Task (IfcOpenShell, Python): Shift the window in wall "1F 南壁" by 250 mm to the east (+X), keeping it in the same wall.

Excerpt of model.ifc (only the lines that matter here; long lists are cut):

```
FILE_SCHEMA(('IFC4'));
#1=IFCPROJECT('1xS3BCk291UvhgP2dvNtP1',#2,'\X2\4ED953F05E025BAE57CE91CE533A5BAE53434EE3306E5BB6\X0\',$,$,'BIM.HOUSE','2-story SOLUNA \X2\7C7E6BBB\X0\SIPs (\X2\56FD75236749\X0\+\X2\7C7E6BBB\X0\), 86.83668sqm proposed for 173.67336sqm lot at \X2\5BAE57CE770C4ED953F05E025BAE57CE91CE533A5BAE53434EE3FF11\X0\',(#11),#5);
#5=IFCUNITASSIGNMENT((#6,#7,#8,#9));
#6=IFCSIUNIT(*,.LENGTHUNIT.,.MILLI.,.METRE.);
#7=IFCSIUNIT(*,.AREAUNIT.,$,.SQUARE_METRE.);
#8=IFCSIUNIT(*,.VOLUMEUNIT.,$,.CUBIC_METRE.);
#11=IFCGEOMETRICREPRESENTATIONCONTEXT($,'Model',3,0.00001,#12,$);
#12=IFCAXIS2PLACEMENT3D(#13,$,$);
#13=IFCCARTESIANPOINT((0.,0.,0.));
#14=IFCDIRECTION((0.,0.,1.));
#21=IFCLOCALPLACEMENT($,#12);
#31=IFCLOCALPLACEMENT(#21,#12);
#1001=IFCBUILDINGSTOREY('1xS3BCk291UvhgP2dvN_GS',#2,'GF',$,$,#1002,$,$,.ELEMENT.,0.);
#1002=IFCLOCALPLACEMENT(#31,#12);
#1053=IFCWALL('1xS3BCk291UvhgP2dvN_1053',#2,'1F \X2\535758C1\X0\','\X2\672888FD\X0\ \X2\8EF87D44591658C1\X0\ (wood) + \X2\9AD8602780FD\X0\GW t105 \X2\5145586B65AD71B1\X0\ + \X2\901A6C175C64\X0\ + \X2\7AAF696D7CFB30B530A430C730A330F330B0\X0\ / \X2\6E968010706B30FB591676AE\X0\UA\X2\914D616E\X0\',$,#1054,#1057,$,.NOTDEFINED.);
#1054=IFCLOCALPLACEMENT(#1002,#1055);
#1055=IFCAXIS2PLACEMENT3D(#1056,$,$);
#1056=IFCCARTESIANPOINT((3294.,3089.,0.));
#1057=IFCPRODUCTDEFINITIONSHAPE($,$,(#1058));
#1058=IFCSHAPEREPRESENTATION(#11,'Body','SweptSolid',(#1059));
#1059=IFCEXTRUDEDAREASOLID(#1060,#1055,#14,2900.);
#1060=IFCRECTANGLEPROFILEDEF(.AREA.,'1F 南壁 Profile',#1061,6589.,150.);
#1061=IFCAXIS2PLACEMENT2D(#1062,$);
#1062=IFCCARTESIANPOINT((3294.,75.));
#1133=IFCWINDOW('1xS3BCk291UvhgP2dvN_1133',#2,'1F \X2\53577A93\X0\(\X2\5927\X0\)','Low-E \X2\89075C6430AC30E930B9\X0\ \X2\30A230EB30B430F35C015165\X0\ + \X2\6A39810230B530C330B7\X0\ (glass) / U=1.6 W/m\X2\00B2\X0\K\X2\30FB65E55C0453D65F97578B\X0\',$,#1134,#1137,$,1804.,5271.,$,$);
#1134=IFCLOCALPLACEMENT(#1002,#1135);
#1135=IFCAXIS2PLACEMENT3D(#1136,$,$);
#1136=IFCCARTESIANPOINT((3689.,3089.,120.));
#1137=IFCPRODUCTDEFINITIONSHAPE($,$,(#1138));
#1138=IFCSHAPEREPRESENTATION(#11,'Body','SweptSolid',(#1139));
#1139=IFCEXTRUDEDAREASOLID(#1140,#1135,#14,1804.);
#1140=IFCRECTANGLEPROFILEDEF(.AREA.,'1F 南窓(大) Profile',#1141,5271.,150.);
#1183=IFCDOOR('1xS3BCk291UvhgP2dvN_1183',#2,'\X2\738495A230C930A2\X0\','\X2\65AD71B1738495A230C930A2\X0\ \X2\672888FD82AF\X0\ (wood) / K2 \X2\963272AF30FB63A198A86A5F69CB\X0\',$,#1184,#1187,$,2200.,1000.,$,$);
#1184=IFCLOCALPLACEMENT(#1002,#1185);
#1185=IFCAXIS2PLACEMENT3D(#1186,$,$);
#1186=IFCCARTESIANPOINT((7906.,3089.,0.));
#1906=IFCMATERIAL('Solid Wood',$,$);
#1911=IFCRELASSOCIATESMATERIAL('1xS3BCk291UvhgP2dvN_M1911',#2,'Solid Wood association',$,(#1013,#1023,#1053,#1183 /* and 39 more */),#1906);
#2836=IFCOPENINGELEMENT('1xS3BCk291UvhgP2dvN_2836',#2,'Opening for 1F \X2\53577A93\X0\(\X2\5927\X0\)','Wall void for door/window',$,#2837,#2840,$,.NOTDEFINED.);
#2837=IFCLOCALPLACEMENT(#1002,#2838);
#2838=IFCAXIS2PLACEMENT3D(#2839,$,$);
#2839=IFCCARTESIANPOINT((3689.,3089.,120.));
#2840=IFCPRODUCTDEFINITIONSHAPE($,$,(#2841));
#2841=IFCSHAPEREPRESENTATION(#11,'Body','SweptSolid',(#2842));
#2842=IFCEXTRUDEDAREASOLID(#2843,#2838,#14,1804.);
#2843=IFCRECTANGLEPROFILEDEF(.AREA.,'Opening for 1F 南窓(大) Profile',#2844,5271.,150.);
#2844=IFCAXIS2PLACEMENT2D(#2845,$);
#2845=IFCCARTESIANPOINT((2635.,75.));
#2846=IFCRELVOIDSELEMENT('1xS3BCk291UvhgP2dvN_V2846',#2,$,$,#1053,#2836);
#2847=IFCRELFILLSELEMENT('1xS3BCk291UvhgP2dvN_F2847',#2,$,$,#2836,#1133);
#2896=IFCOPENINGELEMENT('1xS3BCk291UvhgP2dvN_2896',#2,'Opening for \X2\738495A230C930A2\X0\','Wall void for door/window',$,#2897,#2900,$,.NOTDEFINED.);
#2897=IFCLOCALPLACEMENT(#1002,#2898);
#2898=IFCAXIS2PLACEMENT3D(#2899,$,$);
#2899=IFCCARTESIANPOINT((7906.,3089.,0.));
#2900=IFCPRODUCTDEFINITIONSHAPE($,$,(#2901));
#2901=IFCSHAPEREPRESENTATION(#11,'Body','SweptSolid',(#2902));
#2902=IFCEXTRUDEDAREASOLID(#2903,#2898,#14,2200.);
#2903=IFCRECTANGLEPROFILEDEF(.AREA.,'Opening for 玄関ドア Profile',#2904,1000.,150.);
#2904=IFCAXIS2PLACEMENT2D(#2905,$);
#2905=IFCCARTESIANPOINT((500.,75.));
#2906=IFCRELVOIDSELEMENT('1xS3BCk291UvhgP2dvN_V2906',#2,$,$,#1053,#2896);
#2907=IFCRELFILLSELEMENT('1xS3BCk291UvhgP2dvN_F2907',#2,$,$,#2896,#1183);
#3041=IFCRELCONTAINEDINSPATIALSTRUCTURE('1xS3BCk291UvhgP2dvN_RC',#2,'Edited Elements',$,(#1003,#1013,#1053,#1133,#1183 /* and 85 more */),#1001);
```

```python
import ifcopenshell
import ifcopenshell.api.geometry
import ifcopenshell.util.placement

model = ifcopenshell.open("model.ifc")

window = model.by_guid("1xS3BCk291UvhgP2dvN_1133")
opening = window.FillsVoids[0].RelatingOpeningElement
wall = opening.VoidsElements[0].RelatingBuildingElement

wall_matrix = ifcopenshell.util.placement.get_local_placement(wall.ObjectPlacement)
shift = wall_matrix[:3, 0] * 250.0
before = ifcopenshell.util.placement.get_local_placement(window.ObjectPlacement)[:3, 3].copy()

# The window is not placed relative to its opening, so move both.
for product in (opening, window):
    matrix = ifcopenshell.util.placement.get_local_placement(product.ObjectPlacement)
    matrix[:3, 3] += shift
    ifcopenshell.api.geometry.edit_object_placement(model, product=product, matrix=matrix, is_si=False)

after = ifcopenshell.util.placement.get_local_placement(window.ObjectPlacement)[:3, 3]
print("window moved by", (after - before).round(3) + 0.0)

model.write("model_v2.ifc")
```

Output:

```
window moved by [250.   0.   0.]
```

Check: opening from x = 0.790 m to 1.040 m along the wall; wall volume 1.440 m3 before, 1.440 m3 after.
